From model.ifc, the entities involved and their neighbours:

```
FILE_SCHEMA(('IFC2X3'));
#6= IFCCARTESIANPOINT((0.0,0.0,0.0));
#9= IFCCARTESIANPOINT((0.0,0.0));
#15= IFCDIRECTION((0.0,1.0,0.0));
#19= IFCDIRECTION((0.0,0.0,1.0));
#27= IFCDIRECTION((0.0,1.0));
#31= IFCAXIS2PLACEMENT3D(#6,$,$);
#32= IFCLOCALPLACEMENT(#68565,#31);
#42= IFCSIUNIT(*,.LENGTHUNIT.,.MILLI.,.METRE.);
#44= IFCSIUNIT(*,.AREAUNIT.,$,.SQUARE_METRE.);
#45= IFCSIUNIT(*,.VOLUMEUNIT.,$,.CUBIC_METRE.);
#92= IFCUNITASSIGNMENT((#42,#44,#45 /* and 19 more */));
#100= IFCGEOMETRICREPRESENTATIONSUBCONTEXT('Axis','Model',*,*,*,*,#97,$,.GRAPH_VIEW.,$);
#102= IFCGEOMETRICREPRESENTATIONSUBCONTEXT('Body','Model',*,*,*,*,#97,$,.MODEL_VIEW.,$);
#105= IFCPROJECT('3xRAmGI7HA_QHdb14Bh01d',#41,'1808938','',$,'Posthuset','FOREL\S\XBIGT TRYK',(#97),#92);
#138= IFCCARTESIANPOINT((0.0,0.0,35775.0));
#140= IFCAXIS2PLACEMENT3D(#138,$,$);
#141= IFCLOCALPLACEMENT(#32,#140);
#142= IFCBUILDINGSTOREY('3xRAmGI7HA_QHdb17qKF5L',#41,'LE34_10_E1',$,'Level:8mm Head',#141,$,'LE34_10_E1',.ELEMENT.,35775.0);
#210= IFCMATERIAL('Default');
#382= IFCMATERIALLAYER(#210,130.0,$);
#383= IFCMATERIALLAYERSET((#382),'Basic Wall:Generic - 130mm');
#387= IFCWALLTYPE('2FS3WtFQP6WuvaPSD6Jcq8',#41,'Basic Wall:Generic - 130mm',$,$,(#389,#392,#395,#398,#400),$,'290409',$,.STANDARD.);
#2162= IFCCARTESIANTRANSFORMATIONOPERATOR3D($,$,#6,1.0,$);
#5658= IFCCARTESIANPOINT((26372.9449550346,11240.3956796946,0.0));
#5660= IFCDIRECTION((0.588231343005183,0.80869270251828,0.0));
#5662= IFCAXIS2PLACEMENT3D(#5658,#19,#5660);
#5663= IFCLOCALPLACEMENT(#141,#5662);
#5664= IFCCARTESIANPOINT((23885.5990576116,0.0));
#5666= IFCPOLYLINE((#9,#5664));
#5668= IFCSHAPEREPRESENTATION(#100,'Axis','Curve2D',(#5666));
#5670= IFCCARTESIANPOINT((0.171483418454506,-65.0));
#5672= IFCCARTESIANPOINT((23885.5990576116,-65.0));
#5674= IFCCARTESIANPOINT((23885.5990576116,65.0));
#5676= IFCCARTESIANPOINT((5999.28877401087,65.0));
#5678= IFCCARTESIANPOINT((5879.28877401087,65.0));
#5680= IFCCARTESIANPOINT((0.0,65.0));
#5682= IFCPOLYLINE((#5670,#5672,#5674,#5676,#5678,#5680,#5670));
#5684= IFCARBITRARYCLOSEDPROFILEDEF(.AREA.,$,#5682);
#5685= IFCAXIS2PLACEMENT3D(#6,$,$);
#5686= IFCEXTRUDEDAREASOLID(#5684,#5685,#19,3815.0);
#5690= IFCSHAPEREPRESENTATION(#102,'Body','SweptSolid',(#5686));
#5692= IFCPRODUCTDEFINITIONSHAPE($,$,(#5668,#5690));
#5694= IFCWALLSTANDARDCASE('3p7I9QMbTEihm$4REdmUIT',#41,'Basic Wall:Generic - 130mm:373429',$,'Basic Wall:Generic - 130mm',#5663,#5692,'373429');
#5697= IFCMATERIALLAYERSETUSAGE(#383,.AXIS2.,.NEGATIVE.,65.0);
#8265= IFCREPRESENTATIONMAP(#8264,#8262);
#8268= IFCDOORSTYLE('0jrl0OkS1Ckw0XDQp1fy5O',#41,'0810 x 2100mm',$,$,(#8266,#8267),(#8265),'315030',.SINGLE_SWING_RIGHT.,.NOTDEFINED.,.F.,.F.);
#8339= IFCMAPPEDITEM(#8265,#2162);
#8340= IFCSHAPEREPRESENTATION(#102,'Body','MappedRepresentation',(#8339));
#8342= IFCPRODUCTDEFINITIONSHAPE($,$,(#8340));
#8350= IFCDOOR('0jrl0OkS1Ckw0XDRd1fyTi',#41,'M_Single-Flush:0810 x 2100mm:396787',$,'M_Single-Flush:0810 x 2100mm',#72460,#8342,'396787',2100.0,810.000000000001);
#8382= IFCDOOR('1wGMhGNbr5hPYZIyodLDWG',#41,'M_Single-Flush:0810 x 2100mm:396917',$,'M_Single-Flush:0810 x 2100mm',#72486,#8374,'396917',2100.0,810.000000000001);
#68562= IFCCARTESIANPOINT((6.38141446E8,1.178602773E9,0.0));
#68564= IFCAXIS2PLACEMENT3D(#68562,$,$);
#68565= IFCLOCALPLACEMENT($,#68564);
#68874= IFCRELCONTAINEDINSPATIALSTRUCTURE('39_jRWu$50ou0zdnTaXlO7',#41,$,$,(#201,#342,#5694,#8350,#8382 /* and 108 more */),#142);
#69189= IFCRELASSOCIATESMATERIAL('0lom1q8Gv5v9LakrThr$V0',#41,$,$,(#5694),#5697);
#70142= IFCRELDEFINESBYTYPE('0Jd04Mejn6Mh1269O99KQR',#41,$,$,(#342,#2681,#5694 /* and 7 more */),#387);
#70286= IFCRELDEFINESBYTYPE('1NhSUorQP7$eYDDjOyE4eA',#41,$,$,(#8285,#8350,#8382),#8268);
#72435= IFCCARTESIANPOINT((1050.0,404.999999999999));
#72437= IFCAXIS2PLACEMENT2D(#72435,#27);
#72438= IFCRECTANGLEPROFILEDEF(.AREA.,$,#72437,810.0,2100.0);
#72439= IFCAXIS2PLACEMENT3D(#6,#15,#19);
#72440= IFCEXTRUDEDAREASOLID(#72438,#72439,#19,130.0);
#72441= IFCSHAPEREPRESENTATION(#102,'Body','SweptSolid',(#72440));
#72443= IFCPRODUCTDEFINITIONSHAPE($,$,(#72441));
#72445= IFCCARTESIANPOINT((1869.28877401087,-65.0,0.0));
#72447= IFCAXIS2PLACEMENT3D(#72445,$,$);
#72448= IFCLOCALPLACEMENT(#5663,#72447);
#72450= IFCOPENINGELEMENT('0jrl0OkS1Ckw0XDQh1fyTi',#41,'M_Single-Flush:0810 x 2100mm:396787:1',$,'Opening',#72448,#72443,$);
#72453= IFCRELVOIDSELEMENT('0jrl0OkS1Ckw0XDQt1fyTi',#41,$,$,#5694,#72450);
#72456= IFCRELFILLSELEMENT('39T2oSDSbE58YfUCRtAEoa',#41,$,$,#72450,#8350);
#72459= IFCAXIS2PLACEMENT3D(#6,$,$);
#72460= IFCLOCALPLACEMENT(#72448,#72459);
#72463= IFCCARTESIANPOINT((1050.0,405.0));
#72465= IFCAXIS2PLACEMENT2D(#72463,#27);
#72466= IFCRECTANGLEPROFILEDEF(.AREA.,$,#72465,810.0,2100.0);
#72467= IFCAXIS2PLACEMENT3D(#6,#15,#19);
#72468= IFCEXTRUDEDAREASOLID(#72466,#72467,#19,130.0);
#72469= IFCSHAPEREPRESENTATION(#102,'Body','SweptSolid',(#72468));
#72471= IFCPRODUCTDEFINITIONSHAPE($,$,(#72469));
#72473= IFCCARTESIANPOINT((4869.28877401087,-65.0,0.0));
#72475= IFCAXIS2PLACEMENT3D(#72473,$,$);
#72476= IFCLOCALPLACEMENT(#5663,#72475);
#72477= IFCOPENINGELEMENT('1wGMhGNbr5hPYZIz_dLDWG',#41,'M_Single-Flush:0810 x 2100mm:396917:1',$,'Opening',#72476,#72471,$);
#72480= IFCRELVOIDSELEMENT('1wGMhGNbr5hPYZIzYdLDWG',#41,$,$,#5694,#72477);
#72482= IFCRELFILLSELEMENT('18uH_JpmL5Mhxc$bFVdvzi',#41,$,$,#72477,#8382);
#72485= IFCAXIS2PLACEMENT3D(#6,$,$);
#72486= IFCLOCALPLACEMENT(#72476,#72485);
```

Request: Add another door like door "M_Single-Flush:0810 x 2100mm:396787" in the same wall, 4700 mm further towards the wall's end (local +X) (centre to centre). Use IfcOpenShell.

```python
import ifcopenshell
import ifcopenshell.api.feature
import ifcopenshell.api.geometry
import ifcopenshell.api.root
import ifcopenshell.geom
import ifcopenshell.util.element
import ifcopenshell.util.placement
import ifcopenshell.util.shape

model = ifcopenshell.open("model.ifc")
settings = ifcopenshell.geom.settings()


def volume(element):
    """Net volume in cubic metres, openings subtracted."""
    shape = ifcopenshell.geom.create_shape(settings, element)
    return ifcopenshell.util.shape.get_volume(shape.geometry)


def reuse_history(source, copy):
    """copy_class also copies each property set's owner history, people and application; keep the originals."""
    for rel in copy.IsDefinedBy:
        if rel.is_a("IfcRelDefinesByProperties") and (history := rel.RelatingPropertyDefinition.OwnerHistory):
            rel.RelatingPropertyDefinition.OwnerHistory = source.OwnerHistory
            ifcopenshell.util.element.remove_deep2(model, history)


door = model.by_guid("0jrl0OkS1Ckw0XDRd1fyTi")
opening = door.FillsVoids[0].RelatingOpeningElement
wall = opening.VoidsElements[0].RelatingBuildingElement
before = volume(wall)
shift = ifcopenshell.util.placement.get_local_placement(wall.ObjectPlacement)[:3, 0] * 4700.0

# copy_class copies the void relationship, type, container and properties, but no geometry.
new_opening = ifcopenshell.api.root.copy_class(model, product=opening)
new_opening.Representation = ifcopenshell.util.element.copy_deep(
    model, opening.Representation, exclude=["IfcGeometricRepresentationContext", "IfcRepresentationMap"]
)
new_opening.Name = "M_Single-Flush:0810 x 2100mm"
new_door = ifcopenshell.api.root.copy_class(model, product=door)
new_door.Representation = ifcopenshell.util.element.copy_deep(
    model, door.Representation, exclude=["IfcGeometricRepresentationContext", "IfcRepresentationMap"]
)
new_door.Name = "M_Single-Flush:0810 x 2100mm"
new_door.Tag = None
reuse_history(door, new_door)
fills = ifcopenshell.api.feature.add_filling(model, opening=new_opening, element=new_door)
fills.OwnerHistory = new_door.OwnerHistory  # required in IFC2X3

for old, new in ((opening, new_opening), (door, new_door)):
    matrix = ifcopenshell.util.placement.get_local_placement(old.ObjectPlacement)
    matrix[:3, 3] += shift
    ifcopenshell.api.geometry.edit_object_placement(model, product=new, matrix=matrix, is_si=False)

after = volume(wall)

print(f"wall volume {before:.3f} -> {after:.3f} m3")

model.write("model_edited.ifc")
```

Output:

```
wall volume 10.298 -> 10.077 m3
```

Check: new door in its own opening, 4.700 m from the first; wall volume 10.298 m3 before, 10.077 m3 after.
